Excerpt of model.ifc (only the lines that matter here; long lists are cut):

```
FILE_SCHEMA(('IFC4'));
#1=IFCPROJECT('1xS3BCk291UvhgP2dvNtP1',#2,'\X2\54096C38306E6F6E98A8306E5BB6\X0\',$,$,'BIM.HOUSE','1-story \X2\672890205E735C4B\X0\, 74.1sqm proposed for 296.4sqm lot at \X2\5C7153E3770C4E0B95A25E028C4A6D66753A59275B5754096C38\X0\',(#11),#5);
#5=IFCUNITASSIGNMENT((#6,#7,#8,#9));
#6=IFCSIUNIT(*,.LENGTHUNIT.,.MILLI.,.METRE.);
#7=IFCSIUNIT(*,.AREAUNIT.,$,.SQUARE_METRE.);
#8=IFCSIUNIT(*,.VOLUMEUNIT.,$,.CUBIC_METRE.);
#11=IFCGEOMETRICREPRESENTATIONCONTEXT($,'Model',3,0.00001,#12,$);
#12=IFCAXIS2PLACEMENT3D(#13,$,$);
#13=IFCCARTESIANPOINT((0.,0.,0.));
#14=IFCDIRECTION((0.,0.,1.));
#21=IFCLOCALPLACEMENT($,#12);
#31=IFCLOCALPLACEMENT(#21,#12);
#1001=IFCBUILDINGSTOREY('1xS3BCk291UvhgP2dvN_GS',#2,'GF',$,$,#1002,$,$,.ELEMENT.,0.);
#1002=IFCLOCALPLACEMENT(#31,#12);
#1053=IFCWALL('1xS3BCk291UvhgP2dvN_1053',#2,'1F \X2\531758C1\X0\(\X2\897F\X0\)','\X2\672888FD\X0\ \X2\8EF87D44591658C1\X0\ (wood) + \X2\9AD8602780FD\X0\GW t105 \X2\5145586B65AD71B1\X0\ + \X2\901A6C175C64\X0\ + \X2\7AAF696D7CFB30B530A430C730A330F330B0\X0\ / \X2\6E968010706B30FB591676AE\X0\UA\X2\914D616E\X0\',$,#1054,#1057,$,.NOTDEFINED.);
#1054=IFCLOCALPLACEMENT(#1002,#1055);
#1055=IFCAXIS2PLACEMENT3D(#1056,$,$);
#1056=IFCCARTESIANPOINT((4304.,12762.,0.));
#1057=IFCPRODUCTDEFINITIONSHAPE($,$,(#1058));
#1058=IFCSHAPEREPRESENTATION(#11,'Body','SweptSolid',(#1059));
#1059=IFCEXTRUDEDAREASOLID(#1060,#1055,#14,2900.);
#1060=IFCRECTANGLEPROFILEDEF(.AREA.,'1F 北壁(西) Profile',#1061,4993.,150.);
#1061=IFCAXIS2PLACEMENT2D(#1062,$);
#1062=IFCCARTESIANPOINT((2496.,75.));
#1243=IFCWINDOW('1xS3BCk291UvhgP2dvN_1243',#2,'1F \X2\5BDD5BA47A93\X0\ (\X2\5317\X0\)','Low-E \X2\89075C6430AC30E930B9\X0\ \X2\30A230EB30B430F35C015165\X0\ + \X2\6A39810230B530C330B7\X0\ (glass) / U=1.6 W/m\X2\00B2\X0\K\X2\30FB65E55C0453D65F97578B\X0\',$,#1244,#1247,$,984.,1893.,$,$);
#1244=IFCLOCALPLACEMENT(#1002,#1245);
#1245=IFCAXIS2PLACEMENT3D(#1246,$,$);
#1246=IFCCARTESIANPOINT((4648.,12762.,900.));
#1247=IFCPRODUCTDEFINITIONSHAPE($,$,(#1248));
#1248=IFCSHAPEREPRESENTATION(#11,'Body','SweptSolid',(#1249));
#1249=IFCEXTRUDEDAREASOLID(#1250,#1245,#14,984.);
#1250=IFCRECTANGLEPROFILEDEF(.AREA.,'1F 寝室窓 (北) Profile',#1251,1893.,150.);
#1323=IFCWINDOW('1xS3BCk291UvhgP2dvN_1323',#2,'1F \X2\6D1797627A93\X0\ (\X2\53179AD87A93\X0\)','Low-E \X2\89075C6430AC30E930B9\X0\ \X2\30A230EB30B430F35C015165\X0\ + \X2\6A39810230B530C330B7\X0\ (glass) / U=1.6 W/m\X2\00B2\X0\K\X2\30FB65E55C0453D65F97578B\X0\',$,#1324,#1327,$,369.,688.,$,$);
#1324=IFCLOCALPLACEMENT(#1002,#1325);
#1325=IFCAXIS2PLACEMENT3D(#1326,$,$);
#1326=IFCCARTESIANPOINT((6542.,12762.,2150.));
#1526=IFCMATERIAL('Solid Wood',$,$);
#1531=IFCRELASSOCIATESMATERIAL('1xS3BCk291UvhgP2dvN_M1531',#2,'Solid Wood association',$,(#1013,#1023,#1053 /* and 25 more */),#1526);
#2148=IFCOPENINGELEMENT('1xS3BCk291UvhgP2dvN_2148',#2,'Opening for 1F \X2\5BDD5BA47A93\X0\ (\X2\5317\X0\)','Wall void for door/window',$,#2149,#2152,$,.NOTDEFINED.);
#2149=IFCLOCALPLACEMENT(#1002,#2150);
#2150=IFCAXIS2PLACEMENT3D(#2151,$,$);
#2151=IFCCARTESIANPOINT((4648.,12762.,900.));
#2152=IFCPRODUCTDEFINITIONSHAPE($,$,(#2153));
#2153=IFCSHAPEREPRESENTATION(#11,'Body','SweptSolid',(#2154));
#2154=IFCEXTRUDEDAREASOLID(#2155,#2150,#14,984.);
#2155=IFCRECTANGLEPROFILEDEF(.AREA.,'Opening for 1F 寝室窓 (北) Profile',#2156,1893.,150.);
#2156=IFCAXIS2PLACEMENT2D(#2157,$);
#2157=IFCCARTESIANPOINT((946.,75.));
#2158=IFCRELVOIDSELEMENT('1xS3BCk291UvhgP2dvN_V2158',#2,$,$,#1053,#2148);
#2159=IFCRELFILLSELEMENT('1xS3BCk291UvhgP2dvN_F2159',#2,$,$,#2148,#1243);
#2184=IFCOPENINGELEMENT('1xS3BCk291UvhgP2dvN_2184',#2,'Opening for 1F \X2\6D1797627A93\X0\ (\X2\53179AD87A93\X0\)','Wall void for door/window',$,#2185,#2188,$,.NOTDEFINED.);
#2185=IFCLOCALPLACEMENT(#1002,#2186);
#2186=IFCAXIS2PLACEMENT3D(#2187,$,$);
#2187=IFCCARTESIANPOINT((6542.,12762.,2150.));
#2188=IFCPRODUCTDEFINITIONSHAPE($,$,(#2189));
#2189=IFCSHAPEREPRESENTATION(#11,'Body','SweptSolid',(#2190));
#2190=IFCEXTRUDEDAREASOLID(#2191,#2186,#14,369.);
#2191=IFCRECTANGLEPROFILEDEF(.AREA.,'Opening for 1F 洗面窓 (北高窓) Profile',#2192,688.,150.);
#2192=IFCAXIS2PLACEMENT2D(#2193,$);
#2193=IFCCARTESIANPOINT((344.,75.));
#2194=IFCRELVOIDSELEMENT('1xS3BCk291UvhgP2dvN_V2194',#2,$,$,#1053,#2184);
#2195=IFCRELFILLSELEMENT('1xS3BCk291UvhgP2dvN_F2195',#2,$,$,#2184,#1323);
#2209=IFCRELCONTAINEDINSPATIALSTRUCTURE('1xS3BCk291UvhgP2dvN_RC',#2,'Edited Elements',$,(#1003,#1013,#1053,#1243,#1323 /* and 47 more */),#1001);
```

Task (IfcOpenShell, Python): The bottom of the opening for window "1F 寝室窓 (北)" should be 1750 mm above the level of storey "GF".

```python
import numpy as np
import ifcopenshell
import ifcopenshell.api.geometry
import ifcopenshell.geom
import ifcopenshell.util.element
import ifcopenshell.util.placement
import ifcopenshell.util.shape
import ifcopenshell.util.unit

model = ifcopenshell.open("model.ifc")
unit_scale = ifcopenshell.util.unit.calculate_unit_scale(model)

window = model.by_guid("1xS3BCk291UvhgP2dvN_1243")
opening = window.FillsVoids[0].RelatingOpeningElement
storey = ifcopenshell.util.element.get_container(window, ifc_class="IfcBuildingStorey")
level = ifcopenshell.util.placement.get_local_placement(storey.ObjectPlacement)[2, 3]

# The opening's origin need not be at the sill, so measure its lowest point.
shape = ifcopenshell.geom.create_shape(ifcopenshell.geom.settings(), opening)
bottom = ifcopenshell.util.shape.get_shape_bottom_elevation(shape, shape.geometry) / unit_scale
dz = level + 1750.0 - bottom

shift = np.array([0.0, 0.0, dz])
# The window is not placed relative to its opening, so move both.
for product in (opening, window):
    matrix = ifcopenshell.util.placement.get_local_placement(product.ObjectPlacement)
    matrix[:3, 3] += shift
    ifcopenshell.api.geometry.edit_object_placement(model, product=product, matrix=matrix, is_si=False)

print(f"moved by {dz * unit_scale:+.3f} m")

model.write("model_v2.ifc")
```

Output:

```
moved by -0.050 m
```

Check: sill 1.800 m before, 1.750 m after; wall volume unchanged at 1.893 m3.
